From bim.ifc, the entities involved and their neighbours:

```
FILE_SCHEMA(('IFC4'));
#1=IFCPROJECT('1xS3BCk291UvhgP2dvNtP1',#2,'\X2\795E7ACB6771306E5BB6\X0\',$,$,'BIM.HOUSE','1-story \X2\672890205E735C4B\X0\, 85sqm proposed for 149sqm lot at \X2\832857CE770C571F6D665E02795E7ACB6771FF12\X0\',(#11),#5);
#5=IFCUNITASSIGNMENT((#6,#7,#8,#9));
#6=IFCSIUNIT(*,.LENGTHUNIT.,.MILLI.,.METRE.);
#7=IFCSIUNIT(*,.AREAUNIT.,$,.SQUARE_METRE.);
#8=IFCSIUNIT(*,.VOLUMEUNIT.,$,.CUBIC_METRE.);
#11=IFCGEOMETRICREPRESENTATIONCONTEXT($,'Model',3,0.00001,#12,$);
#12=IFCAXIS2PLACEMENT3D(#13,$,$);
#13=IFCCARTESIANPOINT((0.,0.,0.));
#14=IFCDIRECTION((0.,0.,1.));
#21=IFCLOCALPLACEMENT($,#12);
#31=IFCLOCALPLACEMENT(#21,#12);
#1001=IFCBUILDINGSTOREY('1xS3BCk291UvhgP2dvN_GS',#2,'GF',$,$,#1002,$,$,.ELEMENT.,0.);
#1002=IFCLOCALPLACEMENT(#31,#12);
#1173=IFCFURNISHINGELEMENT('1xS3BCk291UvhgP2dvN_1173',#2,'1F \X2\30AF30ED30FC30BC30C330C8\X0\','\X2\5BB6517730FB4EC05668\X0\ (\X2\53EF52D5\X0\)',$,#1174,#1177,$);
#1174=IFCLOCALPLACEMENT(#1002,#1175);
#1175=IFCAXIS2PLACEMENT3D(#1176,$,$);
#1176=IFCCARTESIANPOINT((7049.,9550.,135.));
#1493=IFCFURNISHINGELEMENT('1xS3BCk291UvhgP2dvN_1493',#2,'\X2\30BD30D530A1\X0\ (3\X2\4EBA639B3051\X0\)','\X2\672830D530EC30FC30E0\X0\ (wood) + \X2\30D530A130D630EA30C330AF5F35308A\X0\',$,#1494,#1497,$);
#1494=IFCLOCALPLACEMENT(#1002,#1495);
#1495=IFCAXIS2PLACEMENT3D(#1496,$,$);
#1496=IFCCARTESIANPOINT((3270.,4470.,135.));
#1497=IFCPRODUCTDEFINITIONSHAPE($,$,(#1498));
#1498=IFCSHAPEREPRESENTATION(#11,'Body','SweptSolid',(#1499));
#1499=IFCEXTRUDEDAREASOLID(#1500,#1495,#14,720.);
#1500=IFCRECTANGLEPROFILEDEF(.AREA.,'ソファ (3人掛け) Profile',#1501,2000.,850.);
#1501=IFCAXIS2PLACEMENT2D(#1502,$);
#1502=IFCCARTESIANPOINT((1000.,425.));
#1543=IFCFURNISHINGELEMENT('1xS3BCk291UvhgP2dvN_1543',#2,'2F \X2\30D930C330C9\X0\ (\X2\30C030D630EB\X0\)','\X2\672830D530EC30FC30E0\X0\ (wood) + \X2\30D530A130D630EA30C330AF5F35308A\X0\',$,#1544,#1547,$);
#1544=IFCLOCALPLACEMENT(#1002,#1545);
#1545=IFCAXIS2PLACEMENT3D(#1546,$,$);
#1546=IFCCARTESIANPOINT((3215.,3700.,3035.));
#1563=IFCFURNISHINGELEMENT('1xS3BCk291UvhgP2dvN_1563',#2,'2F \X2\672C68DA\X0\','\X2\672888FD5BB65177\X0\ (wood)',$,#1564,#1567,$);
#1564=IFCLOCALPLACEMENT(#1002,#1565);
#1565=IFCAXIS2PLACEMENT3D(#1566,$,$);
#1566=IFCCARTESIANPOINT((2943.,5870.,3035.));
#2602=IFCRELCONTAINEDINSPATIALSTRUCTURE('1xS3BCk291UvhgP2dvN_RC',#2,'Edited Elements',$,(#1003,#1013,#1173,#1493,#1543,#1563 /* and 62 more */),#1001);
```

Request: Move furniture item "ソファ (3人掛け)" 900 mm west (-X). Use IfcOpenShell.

```python
import ifcopenshell
import ifcopenshell.api.geometry
import ifcopenshell.util.placement
import ifcopenshell.util.unit

model = ifcopenshell.open("bim.ifc")
unit_scale = ifcopenshell.util.unit.calculate_unit_scale(model)

item = model.by_id(1493)
matrix = ifcopenshell.util.placement.get_local_placement(item.ObjectPlacement)
matrix[0, 3] -= 0.9 / unit_scale
ifcopenshell.api.geometry.edit_object_placement(model, product=item, matrix=matrix, is_si=False)

print(ifcopenshell.util.placement.get_local_placement(item.ObjectPlacement).round(3) + 0.0)

model.write("bim_rev.ifc")
```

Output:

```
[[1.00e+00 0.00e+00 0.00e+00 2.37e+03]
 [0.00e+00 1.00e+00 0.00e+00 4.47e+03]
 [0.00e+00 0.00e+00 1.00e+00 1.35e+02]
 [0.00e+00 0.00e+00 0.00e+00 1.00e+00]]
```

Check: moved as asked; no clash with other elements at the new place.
